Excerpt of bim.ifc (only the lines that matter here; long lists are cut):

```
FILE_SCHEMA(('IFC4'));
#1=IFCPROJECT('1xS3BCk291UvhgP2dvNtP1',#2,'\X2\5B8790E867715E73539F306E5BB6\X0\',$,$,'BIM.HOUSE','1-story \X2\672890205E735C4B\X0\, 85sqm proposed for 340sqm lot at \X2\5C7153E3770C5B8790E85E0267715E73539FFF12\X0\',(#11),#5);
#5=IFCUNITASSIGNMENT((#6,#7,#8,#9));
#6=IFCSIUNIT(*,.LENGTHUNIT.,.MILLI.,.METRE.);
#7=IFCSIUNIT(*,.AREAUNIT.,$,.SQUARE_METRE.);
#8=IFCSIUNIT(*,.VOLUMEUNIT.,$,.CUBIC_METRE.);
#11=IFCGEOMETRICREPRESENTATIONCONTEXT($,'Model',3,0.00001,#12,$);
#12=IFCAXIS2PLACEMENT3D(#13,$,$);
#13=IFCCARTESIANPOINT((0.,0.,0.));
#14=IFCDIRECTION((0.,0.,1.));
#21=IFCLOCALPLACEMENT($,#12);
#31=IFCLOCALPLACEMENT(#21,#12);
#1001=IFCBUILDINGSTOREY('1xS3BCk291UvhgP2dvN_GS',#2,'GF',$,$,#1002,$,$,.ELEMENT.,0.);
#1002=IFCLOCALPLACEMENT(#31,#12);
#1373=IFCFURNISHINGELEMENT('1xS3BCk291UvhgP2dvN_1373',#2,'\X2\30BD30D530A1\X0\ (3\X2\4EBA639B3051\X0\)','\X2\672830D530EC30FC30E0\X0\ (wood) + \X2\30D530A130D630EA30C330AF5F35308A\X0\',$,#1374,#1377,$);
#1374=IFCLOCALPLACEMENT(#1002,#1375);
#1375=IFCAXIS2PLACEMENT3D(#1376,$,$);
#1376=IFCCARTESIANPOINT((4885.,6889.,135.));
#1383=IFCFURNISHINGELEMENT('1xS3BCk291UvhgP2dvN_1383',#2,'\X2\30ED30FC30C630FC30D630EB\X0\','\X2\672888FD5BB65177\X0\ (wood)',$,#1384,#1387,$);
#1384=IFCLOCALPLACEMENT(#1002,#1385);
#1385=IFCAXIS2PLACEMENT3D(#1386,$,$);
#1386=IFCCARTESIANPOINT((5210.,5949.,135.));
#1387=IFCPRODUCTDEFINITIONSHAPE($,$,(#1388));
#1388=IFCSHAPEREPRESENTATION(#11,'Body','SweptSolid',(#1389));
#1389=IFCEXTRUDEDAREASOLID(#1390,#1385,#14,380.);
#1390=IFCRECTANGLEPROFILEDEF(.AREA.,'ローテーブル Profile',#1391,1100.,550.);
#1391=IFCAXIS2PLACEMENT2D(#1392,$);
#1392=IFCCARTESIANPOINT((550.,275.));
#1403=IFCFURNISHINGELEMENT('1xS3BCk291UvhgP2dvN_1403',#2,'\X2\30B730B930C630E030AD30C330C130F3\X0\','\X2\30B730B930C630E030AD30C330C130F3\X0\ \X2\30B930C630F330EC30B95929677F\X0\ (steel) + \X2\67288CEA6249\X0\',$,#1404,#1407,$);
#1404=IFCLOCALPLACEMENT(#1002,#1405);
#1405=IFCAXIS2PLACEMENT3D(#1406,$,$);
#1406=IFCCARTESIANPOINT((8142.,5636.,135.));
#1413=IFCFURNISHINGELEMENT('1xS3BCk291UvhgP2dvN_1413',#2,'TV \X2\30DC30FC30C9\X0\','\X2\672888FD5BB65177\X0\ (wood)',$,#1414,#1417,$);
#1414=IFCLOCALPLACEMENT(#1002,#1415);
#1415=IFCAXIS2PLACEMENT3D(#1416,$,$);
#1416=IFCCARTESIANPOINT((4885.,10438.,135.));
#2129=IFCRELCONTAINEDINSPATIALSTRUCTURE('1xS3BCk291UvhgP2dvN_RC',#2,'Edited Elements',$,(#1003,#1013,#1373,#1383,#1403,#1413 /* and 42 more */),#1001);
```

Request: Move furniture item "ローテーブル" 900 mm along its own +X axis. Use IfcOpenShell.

```python
import ifcopenshell
import ifcopenshell.api.geometry
import ifcopenshell.util.placement
import ifcopenshell.util.unit

model = ifcopenshell.open("bim.ifc")
unit_scale = ifcopenshell.util.unit.calculate_unit_scale(model)

item = model.by_guid("1xS3BCk291UvhgP2dvN_1383")
matrix = ifcopenshell.util.placement.get_local_placement(item.ObjectPlacement)
matrix[:3, 3] += matrix[:3, 0] * 0.9 / unit_scale
ifcopenshell.api.geometry.edit_object_placement(model, product=item, matrix=matrix, is_si=False)

print(ifcopenshell.util.placement.get_local_placement(item.ObjectPlacement).round(3) + 0.0)

model.write("bim_edited.ifc")
```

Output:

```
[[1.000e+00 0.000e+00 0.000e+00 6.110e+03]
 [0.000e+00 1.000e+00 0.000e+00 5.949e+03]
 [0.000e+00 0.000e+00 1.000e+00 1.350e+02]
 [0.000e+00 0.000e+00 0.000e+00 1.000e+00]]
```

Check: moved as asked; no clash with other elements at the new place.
